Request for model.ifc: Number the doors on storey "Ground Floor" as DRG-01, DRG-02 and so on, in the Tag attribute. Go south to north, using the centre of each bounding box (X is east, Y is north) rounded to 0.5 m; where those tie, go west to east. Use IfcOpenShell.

First a look at what the model holds.

```python
import ifcopenshell
import ifcopenshell.util.element
import ifcopenshell.util.placement

model = ifcopenshell.open("model.ifc")
print(model.schema)
storey = next(s for s in model.by_type("IfcBuildingStorey") if s.Name == "Ground Floor")
doors = [e for e in ifcopenshell.util.element.get_decomposition(storey) if e.is_a("IfcDoor")]
for e in sorted(doors, key=lambda e: e.id()):
    origin = ifcopenshell.util.placement.get_local_placement(e.ObjectPlacement)[:3, 3]
    print(e.id(), e.Tag, e.Name, origin.round(2) + 0.0, sep=" | ")
```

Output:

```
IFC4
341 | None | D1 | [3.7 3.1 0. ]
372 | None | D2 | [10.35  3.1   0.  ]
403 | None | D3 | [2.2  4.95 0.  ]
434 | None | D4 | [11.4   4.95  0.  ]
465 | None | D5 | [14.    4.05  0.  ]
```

```python
import ifcopenshell
import ifcopenshell.geom
import ifcopenshell.util.element
import ifcopenshell.util.shape

model = ifcopenshell.open("model.ifc")
settings = ifcopenshell.geom.settings()
settings.set("use-world-coords", True)


def centre(element):
    shape = ifcopenshell.geom.create_shape(settings, element)
    return ifcopenshell.util.shape.get_bbox_centroid(shape.geometry)


storey = next(s for s in model.by_type("IfcBuildingStorey") if s.Name == "Ground Floor")
doors = [e for e in ifcopenshell.util.element.get_decomposition(storey) if e.is_a("IfcDoor")]

# Insertion points can sit at a corner or the storey origin, so sort by the geometry (in metres).
centres = {e: centre(e) for e in doors}
doors.sort(key=lambda e: (round(centres[e][1] / 0.5), centres[e][0]))

for i, e in enumerate(doors, start=1):
    number = f"DRG-{i:02d}"
    e.Tag = number
    print(e.id(), number)

model.write("model_rev.ifc")
```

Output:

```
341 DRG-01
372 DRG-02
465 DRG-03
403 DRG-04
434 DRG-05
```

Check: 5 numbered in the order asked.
